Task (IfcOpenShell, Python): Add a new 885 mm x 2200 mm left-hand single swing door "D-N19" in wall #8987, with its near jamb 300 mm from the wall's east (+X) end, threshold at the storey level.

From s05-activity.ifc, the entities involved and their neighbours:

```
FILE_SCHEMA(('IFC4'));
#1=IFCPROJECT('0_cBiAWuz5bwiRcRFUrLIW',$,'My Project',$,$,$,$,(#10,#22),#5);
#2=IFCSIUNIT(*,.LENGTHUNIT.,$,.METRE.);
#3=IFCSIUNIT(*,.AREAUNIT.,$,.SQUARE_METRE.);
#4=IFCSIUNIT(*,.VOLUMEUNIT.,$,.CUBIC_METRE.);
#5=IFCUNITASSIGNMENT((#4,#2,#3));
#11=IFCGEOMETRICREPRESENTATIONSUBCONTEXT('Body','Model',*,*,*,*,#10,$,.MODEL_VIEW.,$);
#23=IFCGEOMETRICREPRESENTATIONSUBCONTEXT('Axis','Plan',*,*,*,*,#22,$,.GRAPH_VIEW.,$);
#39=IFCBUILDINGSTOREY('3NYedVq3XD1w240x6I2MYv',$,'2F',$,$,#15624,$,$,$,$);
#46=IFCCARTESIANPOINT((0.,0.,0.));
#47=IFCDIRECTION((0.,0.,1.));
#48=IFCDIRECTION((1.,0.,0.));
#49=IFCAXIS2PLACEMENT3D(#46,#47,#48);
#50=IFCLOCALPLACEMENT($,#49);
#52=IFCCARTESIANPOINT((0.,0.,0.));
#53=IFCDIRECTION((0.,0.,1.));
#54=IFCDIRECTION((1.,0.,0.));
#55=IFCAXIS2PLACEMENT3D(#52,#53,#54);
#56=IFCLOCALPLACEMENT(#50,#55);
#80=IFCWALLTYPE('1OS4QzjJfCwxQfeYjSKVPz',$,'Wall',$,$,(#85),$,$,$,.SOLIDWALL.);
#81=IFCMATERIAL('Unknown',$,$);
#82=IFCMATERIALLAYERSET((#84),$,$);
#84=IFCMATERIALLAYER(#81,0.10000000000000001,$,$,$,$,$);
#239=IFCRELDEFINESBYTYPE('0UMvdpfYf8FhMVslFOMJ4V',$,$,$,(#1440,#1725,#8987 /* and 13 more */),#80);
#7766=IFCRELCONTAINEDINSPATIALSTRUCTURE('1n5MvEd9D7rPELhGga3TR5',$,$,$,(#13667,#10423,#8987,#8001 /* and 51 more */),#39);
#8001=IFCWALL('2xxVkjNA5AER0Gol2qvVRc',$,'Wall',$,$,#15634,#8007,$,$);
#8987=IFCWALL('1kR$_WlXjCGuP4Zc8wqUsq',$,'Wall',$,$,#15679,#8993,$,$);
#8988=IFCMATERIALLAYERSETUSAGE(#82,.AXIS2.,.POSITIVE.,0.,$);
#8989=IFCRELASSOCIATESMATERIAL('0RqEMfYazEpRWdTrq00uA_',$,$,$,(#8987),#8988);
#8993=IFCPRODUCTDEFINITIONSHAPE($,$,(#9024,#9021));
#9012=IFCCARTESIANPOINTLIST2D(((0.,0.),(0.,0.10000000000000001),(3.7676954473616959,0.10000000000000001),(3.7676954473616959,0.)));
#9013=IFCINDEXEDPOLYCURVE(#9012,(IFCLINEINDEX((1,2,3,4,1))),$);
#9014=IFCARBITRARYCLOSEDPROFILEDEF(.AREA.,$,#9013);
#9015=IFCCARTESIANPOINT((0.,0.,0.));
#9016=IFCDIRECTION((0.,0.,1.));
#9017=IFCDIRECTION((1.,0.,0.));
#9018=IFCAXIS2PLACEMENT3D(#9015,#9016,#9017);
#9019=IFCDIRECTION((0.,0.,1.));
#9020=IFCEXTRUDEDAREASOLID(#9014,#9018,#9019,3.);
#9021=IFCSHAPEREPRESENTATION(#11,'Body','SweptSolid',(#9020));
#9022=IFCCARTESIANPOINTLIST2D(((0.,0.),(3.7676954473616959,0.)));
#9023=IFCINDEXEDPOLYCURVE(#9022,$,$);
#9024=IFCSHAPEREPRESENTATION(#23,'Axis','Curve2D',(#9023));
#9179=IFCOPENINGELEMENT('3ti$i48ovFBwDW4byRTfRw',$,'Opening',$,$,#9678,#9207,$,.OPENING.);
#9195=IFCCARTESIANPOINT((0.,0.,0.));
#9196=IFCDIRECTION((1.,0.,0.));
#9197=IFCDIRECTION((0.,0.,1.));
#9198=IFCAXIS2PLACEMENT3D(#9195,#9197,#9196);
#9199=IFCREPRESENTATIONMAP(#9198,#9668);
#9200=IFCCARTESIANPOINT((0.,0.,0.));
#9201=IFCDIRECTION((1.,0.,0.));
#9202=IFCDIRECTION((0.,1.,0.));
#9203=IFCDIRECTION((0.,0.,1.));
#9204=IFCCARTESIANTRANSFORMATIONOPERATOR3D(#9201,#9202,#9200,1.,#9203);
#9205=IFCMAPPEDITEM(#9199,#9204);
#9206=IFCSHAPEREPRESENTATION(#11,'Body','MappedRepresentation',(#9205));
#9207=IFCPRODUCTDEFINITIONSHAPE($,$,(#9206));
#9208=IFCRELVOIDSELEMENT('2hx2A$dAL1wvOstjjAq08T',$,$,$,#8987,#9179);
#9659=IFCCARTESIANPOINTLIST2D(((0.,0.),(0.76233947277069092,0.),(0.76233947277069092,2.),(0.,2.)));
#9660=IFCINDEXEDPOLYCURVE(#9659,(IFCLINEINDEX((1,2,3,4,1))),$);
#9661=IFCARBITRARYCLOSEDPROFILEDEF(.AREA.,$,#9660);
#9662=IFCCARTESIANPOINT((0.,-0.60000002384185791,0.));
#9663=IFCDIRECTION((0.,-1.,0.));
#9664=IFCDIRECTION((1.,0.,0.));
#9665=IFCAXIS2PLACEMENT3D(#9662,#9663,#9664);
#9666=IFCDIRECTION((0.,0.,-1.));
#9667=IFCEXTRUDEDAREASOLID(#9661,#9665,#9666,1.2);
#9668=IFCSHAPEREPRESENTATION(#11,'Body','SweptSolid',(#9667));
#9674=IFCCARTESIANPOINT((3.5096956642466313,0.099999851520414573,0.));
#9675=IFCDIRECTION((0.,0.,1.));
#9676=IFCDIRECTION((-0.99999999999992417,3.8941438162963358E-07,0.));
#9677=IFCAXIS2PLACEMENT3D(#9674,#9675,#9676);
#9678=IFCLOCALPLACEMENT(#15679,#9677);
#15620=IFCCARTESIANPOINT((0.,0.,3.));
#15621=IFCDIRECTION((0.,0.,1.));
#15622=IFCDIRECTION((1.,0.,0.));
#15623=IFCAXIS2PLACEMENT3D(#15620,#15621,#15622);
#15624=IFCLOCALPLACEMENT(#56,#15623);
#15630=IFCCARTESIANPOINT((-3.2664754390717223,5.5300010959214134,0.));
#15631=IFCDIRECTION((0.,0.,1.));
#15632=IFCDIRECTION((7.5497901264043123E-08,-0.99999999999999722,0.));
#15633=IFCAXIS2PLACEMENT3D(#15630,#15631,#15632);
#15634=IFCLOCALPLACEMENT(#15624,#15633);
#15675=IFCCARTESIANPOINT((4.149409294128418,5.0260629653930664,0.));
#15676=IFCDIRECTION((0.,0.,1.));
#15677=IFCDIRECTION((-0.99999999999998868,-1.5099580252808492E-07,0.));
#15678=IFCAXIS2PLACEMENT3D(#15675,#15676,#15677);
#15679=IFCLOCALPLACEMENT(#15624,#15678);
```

```python
import numpy as np
import ifcopenshell
import ifcopenshell.api.feature
import ifcopenshell.api.geometry
import ifcopenshell.api.root
import ifcopenshell.api.spatial
import ifcopenshell.geom
import ifcopenshell.util.element
import ifcopenshell.util.placement
import ifcopenshell.util.representation
import ifcopenshell.util.shape
import ifcopenshell.util.unit

model = ifcopenshell.open("s05-activity.ifc")
unit_scale = ifcopenshell.util.unit.calculate_unit_scale(model)
settings = ifcopenshell.geom.settings()


def volume(element):
    """Net volume in cubic metres, openings subtracted."""
    shape = ifcopenshell.geom.create_shape(settings, element)
    return ifcopenshell.util.shape.get_volume(shape.geometry)


wall = model.by_guid("1kR$_WlXjCGuP4Zc8wqUsq")
storey = ifcopenshell.util.element.get_container(wall, ifc_class="IfcBuildingStorey")
context = ifcopenshell.util.representation.get_context(model, "Model", "Body", "MODEL_VIEW")
before = volume(wall)

width, height, from_end, sill = 0.885, 2.2, 0.3, 0.0  # metres

# The wall runs along its own X axis, and the end named is its -X end.
wall_shape = ifcopenshell.geom.create_shape(settings, wall)
x, y, z = ifcopenshell.util.shape.get_vertices(wall_shape.geometry).T
start = x.min() + from_end
face, thickness = float(y.min()), float(y.max() - y.min())
wall_matrix = ifcopenshell.util.placement.get_local_placement(wall.ObjectPlacement)
level = ifcopenshell.util.placement.get_local_placement(storey.ObjectPlacement)[2, 3]


def in_wall(x, y):
    """Placement at x, y metres in the wall's axes, at sill height."""
    matrix = wall_matrix.copy()
    matrix[:, 3] = wall_matrix @ np.array([x / unit_scale, y / unit_scale, 0.0, 1.0])
    matrix[2, 3] = level + sill / unit_scale
    return matrix


# Opening: a box that overshoots both wall faces by 50 mm.
opening = ifcopenshell.api.root.create_entity(model, ifc_class="IfcOpeningElement", predefined_type="OPENING")
box = ifcopenshell.api.geometry.add_wall_representation(
    model, context=context, length=width, height=height, thickness=thickness + 0.1
)
ifcopenshell.api.geometry.assign_representation(model, product=opening, representation=box)
ifcopenshell.api.geometry.edit_object_placement(model, product=opening, matrix=in_wall(start, face - 0.05), is_si=False)
ifcopenshell.api.feature.add_feature(model, feature=opening, element=wall)

door = ifcopenshell.api.root.create_entity(model, ifc_class="IfcDoor", name="D-N19", predefined_type="DOOR")
door.OverallWidth, door.OverallHeight = width / unit_scale, height / unit_scale
door.OperationType = "SINGLE_SWING_LEFT"
body = ifcopenshell.api.geometry.add_door_representation(
    model,
    context=context,
    overall_width=door.OverallWidth,
    overall_height=door.OverallHeight,
    operation_type="SINGLE_SWING_LEFT",
    lining_properties={"LiningDepth": thickness / unit_scale, "ThresholdDepth": thickness / unit_scale},
)
ifcopenshell.api.geometry.assign_representation(model, product=door, representation=body)
ifcopenshell.api.spatial.assign_container(model, products=[door], relating_structure=storey)
ifcopenshell.api.feature.add_filling(model, opening=opening, element=door)

# The lining spans the wall, so the door starts at the wall face.
ifcopenshell.api.geometry.edit_object_placement(model, product=door, matrix=in_wall(start, face), is_si=False)

after = volume(wall)

print(f"wall volume {before:.3f} -> {after:.3f} m3")

model.write("s05-activity_v2.ifc")
```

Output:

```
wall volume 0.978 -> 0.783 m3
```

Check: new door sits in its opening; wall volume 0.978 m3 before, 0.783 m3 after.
